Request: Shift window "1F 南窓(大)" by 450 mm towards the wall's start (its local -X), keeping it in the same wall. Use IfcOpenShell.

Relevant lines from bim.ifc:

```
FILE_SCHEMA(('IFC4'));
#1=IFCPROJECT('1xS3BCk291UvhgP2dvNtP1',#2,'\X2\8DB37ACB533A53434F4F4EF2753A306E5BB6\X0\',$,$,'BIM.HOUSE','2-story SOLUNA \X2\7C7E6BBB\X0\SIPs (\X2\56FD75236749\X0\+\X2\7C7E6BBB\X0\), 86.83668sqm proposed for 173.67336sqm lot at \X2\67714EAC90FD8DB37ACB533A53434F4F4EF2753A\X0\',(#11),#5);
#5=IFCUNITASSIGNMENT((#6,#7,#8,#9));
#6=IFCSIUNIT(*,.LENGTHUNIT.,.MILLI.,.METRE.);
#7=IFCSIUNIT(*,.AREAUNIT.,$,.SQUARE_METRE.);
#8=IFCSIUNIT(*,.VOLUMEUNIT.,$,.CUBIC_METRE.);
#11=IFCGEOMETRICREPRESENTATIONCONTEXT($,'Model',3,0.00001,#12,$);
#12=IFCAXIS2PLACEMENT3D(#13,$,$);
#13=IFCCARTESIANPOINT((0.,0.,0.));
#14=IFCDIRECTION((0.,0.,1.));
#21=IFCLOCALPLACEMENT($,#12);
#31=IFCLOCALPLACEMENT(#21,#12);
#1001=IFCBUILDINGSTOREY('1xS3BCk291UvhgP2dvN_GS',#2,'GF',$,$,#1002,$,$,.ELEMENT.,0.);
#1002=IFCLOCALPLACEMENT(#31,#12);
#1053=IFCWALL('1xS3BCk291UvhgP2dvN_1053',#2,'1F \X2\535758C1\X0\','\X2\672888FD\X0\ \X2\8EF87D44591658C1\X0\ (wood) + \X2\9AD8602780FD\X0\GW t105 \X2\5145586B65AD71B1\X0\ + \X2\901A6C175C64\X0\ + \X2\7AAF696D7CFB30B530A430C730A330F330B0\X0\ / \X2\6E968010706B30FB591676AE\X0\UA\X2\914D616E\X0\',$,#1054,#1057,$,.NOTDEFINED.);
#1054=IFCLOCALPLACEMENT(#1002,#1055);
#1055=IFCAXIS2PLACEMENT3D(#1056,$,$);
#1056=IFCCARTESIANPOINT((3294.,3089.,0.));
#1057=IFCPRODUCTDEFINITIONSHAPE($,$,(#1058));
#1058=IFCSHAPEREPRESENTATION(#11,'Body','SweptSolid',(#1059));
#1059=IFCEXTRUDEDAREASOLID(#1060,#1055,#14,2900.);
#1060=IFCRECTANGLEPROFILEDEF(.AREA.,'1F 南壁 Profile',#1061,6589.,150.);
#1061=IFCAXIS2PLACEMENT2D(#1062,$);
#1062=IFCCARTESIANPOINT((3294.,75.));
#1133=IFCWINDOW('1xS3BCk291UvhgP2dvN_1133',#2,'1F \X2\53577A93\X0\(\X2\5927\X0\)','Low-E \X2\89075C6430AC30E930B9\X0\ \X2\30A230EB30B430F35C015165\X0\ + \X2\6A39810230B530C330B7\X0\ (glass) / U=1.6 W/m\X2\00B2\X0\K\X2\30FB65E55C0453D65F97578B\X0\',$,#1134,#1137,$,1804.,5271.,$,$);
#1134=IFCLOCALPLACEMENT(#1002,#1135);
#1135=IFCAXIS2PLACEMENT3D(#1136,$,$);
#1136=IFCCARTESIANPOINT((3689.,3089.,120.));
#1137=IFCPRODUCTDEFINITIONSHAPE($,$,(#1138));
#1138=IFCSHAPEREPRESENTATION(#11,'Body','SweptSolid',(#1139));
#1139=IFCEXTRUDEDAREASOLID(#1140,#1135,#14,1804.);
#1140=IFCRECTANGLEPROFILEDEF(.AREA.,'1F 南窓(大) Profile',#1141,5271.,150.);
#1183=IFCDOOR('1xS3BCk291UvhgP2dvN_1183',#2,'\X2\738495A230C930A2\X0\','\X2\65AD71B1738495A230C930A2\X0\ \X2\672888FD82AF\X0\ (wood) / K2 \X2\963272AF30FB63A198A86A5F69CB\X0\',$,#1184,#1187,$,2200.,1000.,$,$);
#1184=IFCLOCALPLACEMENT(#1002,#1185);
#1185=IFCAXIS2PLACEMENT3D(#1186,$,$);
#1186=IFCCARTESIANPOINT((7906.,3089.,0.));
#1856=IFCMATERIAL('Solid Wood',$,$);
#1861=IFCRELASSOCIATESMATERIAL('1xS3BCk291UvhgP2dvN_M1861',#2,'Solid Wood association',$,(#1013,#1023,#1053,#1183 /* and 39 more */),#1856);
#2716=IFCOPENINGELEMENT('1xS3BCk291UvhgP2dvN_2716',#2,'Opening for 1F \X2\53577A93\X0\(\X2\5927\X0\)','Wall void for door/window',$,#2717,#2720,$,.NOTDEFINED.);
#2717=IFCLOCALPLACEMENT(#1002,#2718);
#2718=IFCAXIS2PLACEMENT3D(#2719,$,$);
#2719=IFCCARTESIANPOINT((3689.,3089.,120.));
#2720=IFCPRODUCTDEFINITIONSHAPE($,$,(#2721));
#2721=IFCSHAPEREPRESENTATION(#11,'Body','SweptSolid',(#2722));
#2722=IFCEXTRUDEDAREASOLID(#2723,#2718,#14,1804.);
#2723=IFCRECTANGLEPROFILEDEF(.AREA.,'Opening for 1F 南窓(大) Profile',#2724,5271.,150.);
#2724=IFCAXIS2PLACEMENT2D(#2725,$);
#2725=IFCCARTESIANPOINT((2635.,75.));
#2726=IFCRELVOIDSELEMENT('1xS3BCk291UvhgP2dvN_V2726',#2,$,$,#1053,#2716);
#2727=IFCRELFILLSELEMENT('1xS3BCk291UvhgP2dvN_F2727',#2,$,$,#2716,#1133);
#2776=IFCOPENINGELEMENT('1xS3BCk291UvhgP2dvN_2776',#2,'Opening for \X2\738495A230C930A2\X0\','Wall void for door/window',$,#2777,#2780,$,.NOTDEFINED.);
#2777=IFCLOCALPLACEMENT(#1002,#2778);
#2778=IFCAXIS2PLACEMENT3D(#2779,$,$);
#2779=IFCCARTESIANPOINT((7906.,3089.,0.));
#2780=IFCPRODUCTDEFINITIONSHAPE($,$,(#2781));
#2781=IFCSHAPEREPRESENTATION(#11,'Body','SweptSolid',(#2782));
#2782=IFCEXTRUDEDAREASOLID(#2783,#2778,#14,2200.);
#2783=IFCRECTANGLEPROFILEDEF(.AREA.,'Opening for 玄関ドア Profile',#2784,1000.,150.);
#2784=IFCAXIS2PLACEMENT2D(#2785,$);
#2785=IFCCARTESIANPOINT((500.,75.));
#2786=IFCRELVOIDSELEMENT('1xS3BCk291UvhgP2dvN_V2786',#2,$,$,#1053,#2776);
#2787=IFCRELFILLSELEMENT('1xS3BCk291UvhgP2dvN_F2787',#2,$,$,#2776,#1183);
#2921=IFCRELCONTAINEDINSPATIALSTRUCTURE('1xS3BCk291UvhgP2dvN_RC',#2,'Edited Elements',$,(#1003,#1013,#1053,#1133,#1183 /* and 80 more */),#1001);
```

```python
import ifcopenshell
import ifcopenshell.api.geometry
import ifcopenshell.util.placement

model = ifcopenshell.open("bim.ifc")

window = model.by_guid("1xS3BCk291UvhgP2dvN_1133")
opening = window.FillsVoids[0].RelatingOpeningElement
wall = opening.VoidsElements[0].RelatingBuildingElement

wall_matrix = ifcopenshell.util.placement.get_local_placement(wall.ObjectPlacement)
shift = wall_matrix[:3, 0] * -450.0
before = ifcopenshell.util.placement.get_local_placement(window.ObjectPlacement)[:3, 3].copy()

# The window is not placed relative to its opening, so move both.
for product in (opening, window):
    matrix = ifcopenshell.util.placement.get_local_placement(product.ObjectPlacement)
    matrix[:3, 3] += shift
    ifcopenshell.api.geometry.edit_object_placement(model, product=product, matrix=matrix, is_si=False)

after = ifcopenshell.util.placement.get_local_placement(window.ObjectPlacement)[:3, 3]
print("window moved by", (after - before).round(3) + 0.0)

model.write("bim_updated.ifc")
```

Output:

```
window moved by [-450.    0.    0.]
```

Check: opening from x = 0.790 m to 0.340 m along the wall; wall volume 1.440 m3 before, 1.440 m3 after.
